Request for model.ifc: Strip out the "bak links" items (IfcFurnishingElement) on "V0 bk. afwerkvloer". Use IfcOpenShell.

First a look at what the model holds.

```python
import ifcopenshell
import ifcopenshell.util.element

model = ifcopenshell.open("model.ifc")
print(model.schema)
storey = next(s for s in model.by_type("IfcBuildingStorey") if s.Name == "V0 bk. afwerkvloer")
furniture = [e for e in ifcopenshell.util.element.get_decomposition(storey) if e.is_a("IfcFurnishingElement")]
seen = {}
for e in furniture:
    element_type = ifcopenshell.util.element.get_type(e)
    name = element_type.Name if element_type not in (None, e) else None
    seen[name] = seen.get(name, 0) + 1
for name, count in sorted(seen.items(), key=str):
    print(count, "x", name)
```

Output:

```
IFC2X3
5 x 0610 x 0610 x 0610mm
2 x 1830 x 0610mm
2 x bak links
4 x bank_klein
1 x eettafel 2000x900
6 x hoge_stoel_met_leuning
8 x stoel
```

```python
import ifcopenshell
import ifcopenshell.api.root
import ifcopenshell.util.element

model = ifcopenshell.open("model.ifc")

storey = next(s for s in model.by_type("IfcBuildingStorey") if s.Name == "V0 bk. afwerkvloer")
furniture = [e for e in ifcopenshell.util.element.get_decomposition(storey) if e.is_a("IfcFurnishingElement")]
targets = [e for e in furniture if (t := ifcopenshell.util.element.get_type(e)) not in (None, e) and t.Name == "bak links"]

for e in targets:
    ifcopenshell.api.root.remove_product(model, product=e)
print(len(targets), "removed")

model.write("model_rev.ifc")
```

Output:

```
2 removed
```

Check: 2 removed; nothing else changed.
